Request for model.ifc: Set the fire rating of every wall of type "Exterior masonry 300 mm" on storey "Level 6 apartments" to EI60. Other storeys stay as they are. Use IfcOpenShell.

First a look at what the model holds.

```python
import ifcopenshell
import ifcopenshell.util.element

model = ifcopenshell.open("model.ifc")
print(model.schema)
storey = next(s for s in model.by_type("IfcBuildingStorey") if s.Name == "Level 6 apartments")
walls = [e for e in ifcopenshell.util.element.get_decomposition(storey) if e.is_a("IfcWall")]
seen = {}
for e in walls:
    element_type = ifcopenshell.util.element.get_type(e)
    key = (element_type.Name if element_type != e and element_type else None, ifcopenshell.util.element.get_pset(e, "Pset_WallCommon", "FireRating"))
    seen[key] = seen.get(key, 0) + 1
for (name, value), count in sorted(seen.items(), key=str):
    print(count, "x", name, "|", value)
```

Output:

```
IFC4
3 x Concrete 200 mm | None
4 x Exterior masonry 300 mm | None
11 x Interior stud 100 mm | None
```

```python
import ifcopenshell
import ifcopenshell.api.pset
import ifcopenshell.util.element

model = ifcopenshell.open("model.ifc")

storey = next(s for s in model.by_type("IfcBuildingStorey") if s.Name == "Level 6 apartments")
walls = [e for e in ifcopenshell.util.element.get_decomposition(storey) if e.is_a("IfcWall")]

count = 0
for e in walls:
    element_type = ifcopenshell.util.element.get_type(e)
    if element_type in (None, e) or element_type.Name != "Exterior masonry 300 mm":
        continue
    # add_pset returns the element's existing set when there is one.
    pset = ifcopenshell.api.pset.add_pset(model, product=e, name="Pset_WallCommon")
    ifcopenshell.api.pset.edit_pset(model, pset=pset, properties={"FireRating": "EI60"})
    count += 1

print(count, "walls updated")

model.write("model-out.ifc")
```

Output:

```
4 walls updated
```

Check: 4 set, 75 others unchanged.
